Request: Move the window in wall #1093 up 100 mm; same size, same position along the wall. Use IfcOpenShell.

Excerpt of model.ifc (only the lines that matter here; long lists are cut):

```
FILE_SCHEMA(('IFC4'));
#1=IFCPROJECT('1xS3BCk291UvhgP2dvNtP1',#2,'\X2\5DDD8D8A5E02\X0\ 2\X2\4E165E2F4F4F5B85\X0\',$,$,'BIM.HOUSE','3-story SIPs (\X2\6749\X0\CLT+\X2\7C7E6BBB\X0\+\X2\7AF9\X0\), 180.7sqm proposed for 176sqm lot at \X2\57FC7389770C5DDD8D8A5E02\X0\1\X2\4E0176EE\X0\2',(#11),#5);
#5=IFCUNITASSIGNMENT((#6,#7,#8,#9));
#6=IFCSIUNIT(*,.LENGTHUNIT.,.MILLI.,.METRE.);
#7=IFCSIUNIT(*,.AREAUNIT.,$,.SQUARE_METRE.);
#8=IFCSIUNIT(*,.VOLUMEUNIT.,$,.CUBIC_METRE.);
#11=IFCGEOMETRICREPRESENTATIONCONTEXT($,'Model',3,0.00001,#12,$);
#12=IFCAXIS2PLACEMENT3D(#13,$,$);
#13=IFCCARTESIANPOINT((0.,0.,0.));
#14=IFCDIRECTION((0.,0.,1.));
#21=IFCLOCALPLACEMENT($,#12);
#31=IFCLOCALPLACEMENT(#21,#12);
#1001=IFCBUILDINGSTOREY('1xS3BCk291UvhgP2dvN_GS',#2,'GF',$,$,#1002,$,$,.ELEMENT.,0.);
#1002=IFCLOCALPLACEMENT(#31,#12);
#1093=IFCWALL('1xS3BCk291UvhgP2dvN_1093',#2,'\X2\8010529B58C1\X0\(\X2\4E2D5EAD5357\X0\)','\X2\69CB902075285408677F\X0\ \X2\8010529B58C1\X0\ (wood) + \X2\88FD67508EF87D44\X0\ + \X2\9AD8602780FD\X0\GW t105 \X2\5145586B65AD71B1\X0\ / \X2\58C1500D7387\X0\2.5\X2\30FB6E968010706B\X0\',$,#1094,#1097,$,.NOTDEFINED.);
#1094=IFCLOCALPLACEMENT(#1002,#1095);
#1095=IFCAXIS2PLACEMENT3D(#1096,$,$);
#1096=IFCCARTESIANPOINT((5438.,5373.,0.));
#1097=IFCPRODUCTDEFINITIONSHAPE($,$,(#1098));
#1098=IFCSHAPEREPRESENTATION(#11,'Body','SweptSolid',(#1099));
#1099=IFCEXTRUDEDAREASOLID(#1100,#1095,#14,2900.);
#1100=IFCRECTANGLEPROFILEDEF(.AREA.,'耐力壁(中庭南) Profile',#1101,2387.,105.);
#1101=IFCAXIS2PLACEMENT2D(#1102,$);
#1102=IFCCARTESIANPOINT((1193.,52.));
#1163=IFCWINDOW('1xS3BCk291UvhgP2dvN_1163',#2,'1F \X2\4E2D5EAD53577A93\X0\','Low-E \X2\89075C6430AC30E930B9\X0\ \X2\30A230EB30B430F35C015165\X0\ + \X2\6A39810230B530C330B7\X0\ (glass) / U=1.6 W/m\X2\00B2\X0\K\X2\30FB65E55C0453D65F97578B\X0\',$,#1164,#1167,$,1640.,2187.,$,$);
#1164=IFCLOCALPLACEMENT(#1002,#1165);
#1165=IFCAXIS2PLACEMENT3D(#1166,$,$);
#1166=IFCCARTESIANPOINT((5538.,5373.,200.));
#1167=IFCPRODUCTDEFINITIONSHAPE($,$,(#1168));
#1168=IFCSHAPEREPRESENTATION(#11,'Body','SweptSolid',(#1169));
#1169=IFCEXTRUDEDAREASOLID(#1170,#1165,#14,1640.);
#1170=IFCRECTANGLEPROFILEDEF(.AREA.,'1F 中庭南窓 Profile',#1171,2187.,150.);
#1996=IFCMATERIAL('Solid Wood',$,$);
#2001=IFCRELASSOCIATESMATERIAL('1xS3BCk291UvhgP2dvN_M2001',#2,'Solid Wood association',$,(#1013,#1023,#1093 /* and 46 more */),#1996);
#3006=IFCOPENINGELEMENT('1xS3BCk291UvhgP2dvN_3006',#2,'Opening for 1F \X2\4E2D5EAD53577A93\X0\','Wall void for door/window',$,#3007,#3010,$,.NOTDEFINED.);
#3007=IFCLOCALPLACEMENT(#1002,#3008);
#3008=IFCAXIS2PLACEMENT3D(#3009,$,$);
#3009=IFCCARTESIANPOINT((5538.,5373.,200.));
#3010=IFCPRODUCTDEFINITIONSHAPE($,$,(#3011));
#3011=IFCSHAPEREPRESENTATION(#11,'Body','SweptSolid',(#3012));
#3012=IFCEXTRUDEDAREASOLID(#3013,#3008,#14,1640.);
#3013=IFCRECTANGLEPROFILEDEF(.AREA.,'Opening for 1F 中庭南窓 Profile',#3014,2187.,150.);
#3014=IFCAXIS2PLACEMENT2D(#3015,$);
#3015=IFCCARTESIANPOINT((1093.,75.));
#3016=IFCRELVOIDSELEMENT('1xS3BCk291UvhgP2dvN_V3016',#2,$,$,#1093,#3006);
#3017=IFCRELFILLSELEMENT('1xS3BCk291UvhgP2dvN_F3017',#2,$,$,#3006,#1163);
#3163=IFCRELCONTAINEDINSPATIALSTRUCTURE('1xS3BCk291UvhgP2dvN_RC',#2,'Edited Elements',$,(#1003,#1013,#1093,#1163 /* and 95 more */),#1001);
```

```python
import numpy as np
import ifcopenshell
import ifcopenshell.api.geometry
import ifcopenshell.util.placement
import ifcopenshell.util.unit

model = ifcopenshell.open("model.ifc")
unit_scale = ifcopenshell.util.unit.calculate_unit_scale(model)

window = model.by_id(1163)
opening = window.FillsVoids[0].RelatingOpeningElement
dz = 100.0

shift = np.array([0.0, 0.0, dz])
# The window is not placed relative to its opening, so move both.
for product in (opening, window):
    matrix = ifcopenshell.util.placement.get_local_placement(product.ObjectPlacement)
    matrix[:3, 3] += shift
    ifcopenshell.api.geometry.edit_object_placement(model, product=product, matrix=matrix, is_si=False)

print(f"moved by {dz * unit_scale:+.3f} m")

model.write("model_edited.ifc")
```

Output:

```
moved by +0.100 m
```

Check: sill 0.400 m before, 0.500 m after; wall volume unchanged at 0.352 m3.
